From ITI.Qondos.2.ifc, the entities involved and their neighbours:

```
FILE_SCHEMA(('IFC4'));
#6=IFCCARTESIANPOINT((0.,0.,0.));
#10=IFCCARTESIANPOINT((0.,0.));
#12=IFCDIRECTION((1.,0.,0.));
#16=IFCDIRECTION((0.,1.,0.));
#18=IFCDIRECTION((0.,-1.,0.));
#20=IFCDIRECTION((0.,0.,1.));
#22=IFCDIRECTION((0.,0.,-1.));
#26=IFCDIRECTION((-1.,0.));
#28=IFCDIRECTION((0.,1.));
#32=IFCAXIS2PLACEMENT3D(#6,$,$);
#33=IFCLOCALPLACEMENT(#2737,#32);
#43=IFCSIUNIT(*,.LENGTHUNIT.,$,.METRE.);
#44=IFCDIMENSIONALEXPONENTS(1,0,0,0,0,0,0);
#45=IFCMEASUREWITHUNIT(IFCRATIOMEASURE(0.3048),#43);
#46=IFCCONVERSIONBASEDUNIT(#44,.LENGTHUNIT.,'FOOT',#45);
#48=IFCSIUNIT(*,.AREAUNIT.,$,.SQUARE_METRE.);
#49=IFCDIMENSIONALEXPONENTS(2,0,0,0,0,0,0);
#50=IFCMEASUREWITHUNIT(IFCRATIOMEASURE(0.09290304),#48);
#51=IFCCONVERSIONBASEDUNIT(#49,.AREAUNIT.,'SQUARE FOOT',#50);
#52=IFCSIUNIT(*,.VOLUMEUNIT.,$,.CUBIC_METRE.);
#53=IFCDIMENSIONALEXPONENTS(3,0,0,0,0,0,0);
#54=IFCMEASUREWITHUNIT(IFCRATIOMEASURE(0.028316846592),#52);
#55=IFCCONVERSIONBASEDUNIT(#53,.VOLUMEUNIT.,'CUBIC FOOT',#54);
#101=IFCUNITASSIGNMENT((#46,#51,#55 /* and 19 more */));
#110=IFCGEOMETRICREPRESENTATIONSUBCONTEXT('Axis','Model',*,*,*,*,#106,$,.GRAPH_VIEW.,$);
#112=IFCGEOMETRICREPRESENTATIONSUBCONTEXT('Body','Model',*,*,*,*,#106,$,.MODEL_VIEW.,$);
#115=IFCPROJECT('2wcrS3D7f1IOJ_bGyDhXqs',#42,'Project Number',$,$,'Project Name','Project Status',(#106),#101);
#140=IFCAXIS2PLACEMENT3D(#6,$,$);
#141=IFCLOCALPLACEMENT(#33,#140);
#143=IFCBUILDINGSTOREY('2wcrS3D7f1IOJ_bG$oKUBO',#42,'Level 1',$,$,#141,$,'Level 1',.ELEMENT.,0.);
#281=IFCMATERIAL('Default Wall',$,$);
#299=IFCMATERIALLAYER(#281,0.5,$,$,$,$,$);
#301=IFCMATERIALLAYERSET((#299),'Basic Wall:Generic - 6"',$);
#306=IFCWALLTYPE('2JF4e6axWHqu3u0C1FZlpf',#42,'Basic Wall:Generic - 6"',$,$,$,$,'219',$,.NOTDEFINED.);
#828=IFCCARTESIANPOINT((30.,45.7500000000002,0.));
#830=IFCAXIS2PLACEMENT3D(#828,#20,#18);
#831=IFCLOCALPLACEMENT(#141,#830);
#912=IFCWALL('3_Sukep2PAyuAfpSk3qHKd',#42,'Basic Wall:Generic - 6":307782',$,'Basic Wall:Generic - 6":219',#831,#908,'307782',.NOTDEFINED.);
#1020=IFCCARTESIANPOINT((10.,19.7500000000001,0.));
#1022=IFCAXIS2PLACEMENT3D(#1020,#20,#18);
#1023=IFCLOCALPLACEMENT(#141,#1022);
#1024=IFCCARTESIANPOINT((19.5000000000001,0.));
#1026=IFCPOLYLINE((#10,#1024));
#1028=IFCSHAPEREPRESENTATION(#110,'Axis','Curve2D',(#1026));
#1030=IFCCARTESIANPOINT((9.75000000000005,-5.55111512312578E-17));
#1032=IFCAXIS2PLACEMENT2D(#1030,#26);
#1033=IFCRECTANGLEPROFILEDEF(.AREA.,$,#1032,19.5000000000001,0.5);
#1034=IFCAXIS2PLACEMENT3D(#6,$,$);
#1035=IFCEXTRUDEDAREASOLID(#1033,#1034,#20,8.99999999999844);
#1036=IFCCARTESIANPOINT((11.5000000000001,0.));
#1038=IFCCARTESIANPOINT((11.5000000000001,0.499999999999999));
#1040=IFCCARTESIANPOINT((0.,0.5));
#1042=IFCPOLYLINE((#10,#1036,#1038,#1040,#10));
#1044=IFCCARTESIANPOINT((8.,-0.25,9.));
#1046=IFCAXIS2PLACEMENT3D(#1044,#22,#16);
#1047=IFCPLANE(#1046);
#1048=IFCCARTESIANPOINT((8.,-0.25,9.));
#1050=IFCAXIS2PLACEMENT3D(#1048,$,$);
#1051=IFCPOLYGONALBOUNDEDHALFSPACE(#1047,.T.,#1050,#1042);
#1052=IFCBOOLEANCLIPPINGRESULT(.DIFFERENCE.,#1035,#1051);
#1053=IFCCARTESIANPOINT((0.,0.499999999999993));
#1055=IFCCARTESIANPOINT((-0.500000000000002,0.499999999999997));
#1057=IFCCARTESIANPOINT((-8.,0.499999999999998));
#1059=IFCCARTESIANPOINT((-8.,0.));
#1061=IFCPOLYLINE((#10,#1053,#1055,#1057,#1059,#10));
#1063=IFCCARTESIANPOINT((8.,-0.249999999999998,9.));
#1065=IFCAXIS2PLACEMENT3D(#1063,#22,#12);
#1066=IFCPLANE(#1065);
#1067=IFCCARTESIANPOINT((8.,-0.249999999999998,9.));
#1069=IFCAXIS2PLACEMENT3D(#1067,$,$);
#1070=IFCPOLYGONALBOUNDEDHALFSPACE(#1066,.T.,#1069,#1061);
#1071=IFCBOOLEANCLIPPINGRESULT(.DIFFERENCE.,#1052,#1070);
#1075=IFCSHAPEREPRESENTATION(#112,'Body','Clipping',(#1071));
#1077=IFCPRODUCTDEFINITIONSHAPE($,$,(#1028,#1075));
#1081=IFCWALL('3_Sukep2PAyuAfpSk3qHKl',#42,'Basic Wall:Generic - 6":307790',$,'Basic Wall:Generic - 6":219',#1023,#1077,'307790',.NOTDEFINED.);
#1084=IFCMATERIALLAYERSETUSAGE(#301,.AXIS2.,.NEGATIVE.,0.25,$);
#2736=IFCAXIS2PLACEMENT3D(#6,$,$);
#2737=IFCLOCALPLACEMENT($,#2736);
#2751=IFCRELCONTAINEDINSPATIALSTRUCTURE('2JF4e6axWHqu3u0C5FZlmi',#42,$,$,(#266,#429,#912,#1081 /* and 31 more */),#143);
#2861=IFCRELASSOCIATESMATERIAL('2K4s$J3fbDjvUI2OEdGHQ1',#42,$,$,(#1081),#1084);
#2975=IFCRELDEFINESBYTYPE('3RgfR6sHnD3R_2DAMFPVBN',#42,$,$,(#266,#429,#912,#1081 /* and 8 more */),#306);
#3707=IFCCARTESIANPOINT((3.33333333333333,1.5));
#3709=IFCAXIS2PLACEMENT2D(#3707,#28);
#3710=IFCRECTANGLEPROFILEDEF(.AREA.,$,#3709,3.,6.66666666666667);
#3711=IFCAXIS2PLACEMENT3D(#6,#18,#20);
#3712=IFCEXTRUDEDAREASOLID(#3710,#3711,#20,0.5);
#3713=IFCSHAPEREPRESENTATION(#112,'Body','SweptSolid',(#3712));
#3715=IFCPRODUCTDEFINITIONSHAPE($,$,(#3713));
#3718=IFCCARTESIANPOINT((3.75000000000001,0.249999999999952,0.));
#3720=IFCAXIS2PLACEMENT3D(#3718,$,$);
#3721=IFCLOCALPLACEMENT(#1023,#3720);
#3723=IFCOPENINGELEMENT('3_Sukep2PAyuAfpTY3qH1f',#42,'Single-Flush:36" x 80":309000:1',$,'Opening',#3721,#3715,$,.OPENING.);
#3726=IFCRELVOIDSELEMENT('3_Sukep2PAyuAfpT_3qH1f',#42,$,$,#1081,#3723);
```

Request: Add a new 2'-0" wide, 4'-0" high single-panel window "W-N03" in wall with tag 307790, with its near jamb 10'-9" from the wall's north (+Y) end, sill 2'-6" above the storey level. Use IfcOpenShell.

```python
import numpy as np
import ifcopenshell
import ifcopenshell.api.feature
import ifcopenshell.api.geometry
import ifcopenshell.api.root
import ifcopenshell.api.spatial
import ifcopenshell.geom
import ifcopenshell.util.element
import ifcopenshell.util.placement
import ifcopenshell.util.representation
import ifcopenshell.util.shape
import ifcopenshell.util.unit

model = ifcopenshell.open("ITI.Qondos.2.ifc")
unit_scale = ifcopenshell.util.unit.calculate_unit_scale(model)
settings = ifcopenshell.geom.settings()


def volume(element):
    """Net volume in cubic metres, openings subtracted."""
    shape = ifcopenshell.geom.create_shape(settings, element)
    return ifcopenshell.util.shape.get_volume(shape.geometry)


wall = model.by_guid("3_Sukep2PAyuAfpSk3qHKl")
storey = ifcopenshell.util.element.get_container(wall, ifc_class="IfcBuildingStorey")
context = ifcopenshell.util.representation.get_context(model, "Model", "Body", "MODEL_VIEW")
before = volume(wall)

width, height, from_end, sill = 0.6096, 1.2192, 3.2766, 0.762  # metres

# The wall runs along its own X axis, and the end named is its -X end.
wall_shape = ifcopenshell.geom.create_shape(settings, wall)
x, y, z = ifcopenshell.util.shape.get_vertices(wall_shape.geometry).T
start = x.min() + from_end
face, thickness = float(y.min()), float(y.max() - y.min())
wall_matrix = ifcopenshell.util.placement.get_local_placement(wall.ObjectPlacement)
level = ifcopenshell.util.placement.get_local_placement(storey.ObjectPlacement)[2, 3]


def in_wall(x, y):
    """Placement at x, y metres in the wall's axes, at sill height."""
    matrix = wall_matrix.copy()
    matrix[:, 3] = wall_matrix @ np.array([x / unit_scale, y / unit_scale, 0.0, 1.0])
    matrix[2, 3] = level + sill / unit_scale
    return matrix


# Opening: a box that overshoots both wall faces by 50 mm.
opening = ifcopenshell.api.root.create_entity(model, ifc_class="IfcOpeningElement", predefined_type="OPENING")
box = ifcopenshell.api.geometry.add_wall_representation(
    model, context=context, length=width, height=height, thickness=thickness + 0.1
)
ifcopenshell.api.geometry.assign_representation(model, product=opening, representation=box)
ifcopenshell.api.geometry.edit_object_placement(model, product=opening, matrix=in_wall(start, face - 0.05), is_si=False)
ifcopenshell.api.feature.add_feature(model, feature=opening, element=wall)

window = ifcopenshell.api.root.create_entity(model, ifc_class="IfcWindow", name="W-N03", predefined_type="WINDOW")
window.OverallWidth, window.OverallHeight = width / unit_scale, height / unit_scale
window.PartitioningType = "SINGLE_PANEL"
body = ifcopenshell.api.geometry.add_window_representation(
    model,
    context=context,
    overall_width=window.OverallWidth,
    overall_height=window.OverallHeight,
    partition_type="SINGLE_PANEL",
)
ifcopenshell.api.geometry.assign_representation(model, product=window, representation=body)
ifcopenshell.api.spatial.assign_container(model, products=[window], relating_structure=storey)
ifcopenshell.api.feature.add_filling(model, opening=opening, element=window)

# Centre the window in the wall's thickness.
ifcopenshell.api.geometry.edit_object_placement(model, product=window, matrix=in_wall(start, face), is_si=False)
window_shape = ifcopenshell.geom.create_shape(settings, window)
depth = ifcopenshell.util.shape.get_vertices(window_shape.geometry)[:, 1]
offset = face + thickness / 2 - (depth.min() + depth.max()) / 2
ifcopenshell.api.geometry.edit_object_placement(model, product=window, matrix=in_wall(start, offset), is_si=False)

after = volume(wall)

print(f"wall volume {before:.3f} -> {after:.3f} m3")

model.write("ITI.Qondos.2-out.ifc")
```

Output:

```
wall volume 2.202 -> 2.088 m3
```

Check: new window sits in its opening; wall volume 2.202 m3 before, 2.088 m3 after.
